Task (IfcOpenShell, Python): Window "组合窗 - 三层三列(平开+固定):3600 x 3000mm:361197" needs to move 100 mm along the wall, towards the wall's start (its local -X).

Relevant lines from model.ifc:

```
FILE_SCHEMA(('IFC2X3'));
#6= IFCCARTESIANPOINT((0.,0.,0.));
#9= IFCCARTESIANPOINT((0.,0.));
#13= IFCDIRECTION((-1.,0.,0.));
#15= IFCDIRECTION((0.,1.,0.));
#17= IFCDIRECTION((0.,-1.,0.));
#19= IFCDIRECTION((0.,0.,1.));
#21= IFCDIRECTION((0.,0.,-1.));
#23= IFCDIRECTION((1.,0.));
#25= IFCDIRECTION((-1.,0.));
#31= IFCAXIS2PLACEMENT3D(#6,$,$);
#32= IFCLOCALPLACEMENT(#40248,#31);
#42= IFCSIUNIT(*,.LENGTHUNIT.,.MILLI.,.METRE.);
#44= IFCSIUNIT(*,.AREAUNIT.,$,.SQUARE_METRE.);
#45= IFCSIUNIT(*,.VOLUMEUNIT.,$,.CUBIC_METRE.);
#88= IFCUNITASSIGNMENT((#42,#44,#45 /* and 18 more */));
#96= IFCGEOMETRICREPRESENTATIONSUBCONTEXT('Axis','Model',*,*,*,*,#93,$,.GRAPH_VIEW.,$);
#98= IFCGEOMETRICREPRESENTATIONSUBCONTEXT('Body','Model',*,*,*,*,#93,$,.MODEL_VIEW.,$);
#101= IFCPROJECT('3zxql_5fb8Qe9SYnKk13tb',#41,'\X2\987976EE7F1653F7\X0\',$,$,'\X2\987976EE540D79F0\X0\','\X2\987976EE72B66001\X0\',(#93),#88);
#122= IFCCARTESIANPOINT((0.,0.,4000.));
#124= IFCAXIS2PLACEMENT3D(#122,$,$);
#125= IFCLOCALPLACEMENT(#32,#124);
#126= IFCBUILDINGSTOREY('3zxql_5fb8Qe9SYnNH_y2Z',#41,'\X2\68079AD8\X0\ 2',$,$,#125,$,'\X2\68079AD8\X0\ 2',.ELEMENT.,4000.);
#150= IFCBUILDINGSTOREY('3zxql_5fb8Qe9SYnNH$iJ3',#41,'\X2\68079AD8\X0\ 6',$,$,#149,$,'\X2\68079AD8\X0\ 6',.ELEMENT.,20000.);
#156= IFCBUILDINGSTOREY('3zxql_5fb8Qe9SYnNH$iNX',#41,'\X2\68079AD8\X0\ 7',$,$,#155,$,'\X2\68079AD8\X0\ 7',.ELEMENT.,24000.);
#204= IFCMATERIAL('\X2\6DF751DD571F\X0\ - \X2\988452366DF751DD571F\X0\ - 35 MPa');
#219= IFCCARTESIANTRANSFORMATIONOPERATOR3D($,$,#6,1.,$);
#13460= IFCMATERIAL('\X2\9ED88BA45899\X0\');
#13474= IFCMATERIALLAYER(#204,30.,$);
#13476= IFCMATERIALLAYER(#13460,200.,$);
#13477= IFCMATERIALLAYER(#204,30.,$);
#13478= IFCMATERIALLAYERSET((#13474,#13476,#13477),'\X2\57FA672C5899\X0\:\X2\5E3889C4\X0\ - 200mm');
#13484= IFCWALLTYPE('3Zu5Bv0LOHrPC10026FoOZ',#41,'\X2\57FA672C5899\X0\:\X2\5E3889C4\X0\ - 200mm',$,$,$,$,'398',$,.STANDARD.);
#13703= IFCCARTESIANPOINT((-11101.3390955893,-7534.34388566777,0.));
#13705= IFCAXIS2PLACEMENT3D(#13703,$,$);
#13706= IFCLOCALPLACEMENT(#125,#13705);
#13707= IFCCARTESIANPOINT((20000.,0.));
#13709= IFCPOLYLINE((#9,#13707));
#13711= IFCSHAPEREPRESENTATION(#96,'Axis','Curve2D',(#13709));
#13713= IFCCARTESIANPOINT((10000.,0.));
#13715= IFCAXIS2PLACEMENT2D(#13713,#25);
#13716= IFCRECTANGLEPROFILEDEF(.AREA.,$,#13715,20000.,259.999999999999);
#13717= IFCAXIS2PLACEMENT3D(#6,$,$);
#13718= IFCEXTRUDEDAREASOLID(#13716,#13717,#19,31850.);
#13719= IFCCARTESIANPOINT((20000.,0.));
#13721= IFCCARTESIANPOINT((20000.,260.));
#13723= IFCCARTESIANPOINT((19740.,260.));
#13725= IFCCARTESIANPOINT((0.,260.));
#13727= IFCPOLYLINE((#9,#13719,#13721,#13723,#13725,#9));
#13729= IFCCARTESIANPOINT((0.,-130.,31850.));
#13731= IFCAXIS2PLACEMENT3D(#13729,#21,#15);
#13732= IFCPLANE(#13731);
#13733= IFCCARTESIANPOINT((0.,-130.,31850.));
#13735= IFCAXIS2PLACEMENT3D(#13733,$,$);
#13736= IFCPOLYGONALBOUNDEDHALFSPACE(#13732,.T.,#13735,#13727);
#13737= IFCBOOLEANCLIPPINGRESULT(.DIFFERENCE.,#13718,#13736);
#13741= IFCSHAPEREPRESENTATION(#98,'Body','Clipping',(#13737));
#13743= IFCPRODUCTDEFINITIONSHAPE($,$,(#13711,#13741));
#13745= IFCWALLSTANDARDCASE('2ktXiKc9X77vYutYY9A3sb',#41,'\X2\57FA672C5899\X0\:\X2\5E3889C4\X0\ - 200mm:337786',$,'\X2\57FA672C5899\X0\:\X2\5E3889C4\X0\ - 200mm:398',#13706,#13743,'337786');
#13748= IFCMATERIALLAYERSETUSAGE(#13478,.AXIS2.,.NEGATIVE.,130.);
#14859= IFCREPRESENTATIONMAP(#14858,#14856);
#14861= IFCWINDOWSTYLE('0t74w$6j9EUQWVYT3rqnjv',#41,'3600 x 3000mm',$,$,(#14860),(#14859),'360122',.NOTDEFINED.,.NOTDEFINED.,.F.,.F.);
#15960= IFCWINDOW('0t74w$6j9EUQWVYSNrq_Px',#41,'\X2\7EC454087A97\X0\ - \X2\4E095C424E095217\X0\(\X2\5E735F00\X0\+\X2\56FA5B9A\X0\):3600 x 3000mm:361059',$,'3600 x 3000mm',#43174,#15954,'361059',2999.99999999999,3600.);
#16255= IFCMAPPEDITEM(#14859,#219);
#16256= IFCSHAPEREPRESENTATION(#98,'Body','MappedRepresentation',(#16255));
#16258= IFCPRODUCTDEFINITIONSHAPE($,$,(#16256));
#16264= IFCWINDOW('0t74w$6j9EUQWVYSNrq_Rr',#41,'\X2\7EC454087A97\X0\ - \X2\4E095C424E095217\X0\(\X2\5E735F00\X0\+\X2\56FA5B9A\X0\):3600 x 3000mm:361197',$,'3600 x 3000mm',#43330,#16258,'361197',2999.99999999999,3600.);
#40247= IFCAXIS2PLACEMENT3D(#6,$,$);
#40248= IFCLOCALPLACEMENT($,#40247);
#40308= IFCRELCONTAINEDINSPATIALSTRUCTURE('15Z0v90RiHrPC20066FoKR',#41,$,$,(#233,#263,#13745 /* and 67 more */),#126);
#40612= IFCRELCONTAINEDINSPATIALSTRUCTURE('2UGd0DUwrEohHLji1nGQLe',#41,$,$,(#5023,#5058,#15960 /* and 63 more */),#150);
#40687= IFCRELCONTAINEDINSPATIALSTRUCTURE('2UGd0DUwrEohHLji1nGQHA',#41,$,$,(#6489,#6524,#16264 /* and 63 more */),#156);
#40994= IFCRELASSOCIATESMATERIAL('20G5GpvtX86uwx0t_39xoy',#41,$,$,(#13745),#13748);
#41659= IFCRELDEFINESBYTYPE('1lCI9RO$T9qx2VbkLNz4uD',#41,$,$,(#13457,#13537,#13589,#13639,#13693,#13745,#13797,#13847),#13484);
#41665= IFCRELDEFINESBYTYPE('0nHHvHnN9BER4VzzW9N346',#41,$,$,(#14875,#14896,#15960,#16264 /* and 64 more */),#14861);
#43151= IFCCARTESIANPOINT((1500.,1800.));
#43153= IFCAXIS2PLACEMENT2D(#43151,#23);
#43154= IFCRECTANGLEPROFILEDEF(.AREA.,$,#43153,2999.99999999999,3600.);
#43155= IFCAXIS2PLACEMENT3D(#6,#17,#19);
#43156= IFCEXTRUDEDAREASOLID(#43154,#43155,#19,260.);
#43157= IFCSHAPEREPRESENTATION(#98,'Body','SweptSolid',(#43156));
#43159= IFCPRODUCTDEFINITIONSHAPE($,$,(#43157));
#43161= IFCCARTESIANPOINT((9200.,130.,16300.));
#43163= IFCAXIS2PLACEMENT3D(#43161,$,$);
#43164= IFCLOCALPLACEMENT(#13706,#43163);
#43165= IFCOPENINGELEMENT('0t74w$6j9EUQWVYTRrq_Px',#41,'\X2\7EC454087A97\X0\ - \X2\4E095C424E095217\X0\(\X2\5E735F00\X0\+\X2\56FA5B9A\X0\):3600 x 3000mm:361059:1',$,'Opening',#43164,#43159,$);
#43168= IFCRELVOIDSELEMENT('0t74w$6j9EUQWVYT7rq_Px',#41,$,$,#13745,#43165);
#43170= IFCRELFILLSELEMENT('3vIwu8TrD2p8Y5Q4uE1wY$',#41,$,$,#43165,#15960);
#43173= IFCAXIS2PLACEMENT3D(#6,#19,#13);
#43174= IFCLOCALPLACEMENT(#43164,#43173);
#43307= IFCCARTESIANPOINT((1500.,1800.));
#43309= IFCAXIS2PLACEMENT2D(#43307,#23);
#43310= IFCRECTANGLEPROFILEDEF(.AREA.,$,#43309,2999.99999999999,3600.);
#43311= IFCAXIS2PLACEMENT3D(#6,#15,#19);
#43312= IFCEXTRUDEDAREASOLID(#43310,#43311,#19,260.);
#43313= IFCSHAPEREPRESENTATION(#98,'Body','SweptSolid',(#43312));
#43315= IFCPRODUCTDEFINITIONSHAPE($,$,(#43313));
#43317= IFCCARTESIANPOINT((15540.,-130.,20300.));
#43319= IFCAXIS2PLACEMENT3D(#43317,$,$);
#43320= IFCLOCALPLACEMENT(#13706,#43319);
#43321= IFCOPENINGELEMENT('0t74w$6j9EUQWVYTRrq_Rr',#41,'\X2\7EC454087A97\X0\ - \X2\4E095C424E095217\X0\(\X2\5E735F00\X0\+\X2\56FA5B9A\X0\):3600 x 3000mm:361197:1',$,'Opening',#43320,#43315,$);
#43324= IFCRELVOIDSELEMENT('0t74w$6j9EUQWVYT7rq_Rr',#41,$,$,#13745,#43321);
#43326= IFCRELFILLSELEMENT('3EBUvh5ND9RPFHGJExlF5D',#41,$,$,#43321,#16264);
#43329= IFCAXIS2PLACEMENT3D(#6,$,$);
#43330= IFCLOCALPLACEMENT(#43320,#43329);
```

```python
import ifcopenshell
import ifcopenshell.api.geometry
import ifcopenshell.util.placement
import ifcopenshell.util.unit

model = ifcopenshell.open("model.ifc")
unit_scale = ifcopenshell.util.unit.calculate_unit_scale(model)

window = model.by_guid("0t74w$6j9EUQWVYSNrq_Rr")
opening = window.FillsVoids[0].RelatingOpeningElement
wall = opening.VoidsElements[0].RelatingBuildingElement

wall_matrix = ifcopenshell.util.placement.get_local_placement(wall.ObjectPlacement)
shift = wall_matrix[:3, 0] * -0.1 / unit_scale
before = ifcopenshell.util.placement.get_local_placement(window.ObjectPlacement)[:3, 3].copy()

# The window is placed relative to its opening, so it follows when the opening moves.
matrix = ifcopenshell.util.placement.get_local_placement(opening.ObjectPlacement)
matrix[:3, 3] += shift
ifcopenshell.api.geometry.edit_object_placement(
    model, product=opening, matrix=matrix, is_si=False, should_transform_children=True
)

after = ifcopenshell.util.placement.get_local_placement(window.ObjectPlacement)[:3, 3]
print("window moved by", (after - before).round(3) + 0.0)

model.write("model_rev.ifc")
```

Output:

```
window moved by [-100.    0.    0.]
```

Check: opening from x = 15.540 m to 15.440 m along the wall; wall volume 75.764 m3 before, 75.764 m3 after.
